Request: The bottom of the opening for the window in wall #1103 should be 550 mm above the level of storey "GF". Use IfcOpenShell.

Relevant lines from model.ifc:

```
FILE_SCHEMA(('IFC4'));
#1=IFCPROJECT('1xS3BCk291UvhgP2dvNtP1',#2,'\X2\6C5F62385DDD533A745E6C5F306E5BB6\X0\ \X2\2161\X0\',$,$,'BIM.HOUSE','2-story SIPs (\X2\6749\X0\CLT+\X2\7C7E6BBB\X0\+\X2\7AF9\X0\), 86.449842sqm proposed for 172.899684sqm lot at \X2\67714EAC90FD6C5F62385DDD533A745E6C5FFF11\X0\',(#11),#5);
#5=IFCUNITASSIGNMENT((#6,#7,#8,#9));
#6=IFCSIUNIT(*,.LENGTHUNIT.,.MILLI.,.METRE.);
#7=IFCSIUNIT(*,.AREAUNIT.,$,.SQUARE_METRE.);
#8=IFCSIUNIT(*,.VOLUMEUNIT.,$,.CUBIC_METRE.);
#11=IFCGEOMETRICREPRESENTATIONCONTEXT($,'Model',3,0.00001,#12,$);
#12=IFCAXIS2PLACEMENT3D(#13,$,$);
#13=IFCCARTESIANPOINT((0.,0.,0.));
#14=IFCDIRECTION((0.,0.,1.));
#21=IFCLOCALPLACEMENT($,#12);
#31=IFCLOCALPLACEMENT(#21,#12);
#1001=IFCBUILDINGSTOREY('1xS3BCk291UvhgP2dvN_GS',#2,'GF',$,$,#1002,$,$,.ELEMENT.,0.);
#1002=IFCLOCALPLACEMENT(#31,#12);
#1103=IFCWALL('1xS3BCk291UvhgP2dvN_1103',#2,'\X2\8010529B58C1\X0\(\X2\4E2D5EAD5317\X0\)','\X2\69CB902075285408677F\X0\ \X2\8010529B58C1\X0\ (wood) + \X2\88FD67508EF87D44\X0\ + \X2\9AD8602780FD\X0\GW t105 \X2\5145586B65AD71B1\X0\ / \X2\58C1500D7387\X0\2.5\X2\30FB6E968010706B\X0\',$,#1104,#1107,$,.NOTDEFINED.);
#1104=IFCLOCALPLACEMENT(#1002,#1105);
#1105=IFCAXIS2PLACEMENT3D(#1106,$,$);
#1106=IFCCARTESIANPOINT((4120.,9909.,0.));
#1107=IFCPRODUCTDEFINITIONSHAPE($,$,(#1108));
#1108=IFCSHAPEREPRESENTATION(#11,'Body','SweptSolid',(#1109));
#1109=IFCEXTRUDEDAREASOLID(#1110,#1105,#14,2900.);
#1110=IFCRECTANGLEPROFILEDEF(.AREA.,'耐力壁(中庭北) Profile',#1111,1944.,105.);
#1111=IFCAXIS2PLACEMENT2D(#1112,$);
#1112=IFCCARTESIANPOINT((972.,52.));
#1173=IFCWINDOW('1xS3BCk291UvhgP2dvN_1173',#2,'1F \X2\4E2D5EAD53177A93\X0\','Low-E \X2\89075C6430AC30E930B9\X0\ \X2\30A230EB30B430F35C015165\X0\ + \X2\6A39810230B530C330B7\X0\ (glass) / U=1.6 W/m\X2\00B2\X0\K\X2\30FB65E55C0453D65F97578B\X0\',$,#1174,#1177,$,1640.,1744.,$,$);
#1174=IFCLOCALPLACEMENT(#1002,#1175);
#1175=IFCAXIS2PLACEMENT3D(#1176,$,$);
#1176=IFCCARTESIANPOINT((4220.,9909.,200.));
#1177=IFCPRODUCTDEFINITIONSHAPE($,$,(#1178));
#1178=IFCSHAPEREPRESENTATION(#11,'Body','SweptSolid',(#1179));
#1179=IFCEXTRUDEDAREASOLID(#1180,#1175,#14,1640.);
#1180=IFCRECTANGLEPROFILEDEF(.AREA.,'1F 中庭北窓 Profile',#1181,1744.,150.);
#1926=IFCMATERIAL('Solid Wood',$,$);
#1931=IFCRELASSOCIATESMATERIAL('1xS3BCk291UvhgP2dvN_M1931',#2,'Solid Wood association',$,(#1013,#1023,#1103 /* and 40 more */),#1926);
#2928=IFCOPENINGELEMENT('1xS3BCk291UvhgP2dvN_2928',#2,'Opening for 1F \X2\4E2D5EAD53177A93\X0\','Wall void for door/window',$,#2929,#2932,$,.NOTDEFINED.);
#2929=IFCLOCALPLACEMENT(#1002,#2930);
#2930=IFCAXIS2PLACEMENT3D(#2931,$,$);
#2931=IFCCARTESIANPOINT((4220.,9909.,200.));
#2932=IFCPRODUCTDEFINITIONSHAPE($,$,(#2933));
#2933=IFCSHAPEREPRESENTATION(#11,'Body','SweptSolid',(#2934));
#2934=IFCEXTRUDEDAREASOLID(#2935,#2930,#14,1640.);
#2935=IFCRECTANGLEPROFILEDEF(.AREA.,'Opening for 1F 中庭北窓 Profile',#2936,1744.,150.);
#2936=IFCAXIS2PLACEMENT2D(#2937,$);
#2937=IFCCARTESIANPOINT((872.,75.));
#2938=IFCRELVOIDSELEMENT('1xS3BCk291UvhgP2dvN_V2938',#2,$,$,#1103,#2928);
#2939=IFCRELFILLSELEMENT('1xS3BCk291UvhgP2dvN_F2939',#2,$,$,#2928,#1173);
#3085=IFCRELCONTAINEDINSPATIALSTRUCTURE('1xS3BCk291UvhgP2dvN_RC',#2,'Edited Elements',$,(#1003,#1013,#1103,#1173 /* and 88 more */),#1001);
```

```python
import numpy as np
import ifcopenshell
import ifcopenshell.api.geometry
import ifcopenshell.geom
import ifcopenshell.util.element
import ifcopenshell.util.placement
import ifcopenshell.util.shape
import ifcopenshell.util.unit

model = ifcopenshell.open("model.ifc")
unit_scale = ifcopenshell.util.unit.calculate_unit_scale(model)

window = model.by_guid("1xS3BCk291UvhgP2dvN_1173")
opening = window.FillsVoids[0].RelatingOpeningElement
storey = ifcopenshell.util.element.get_container(window, ifc_class="IfcBuildingStorey")
level = ifcopenshell.util.placement.get_local_placement(storey.ObjectPlacement)[2, 3]

# The opening's origin need not be at the sill, so measure its lowest point.
shape = ifcopenshell.geom.create_shape(ifcopenshell.geom.settings(), opening)
bottom = ifcopenshell.util.shape.get_shape_bottom_elevation(shape, shape.geometry) / unit_scale
dz = level + 0.55 / unit_scale - bottom

shift = np.array([0.0, 0.0, dz])
# The window is not placed relative to its opening, so move both.
for product in (opening, window):
    matrix = ifcopenshell.util.placement.get_local_placement(product.ObjectPlacement)
    matrix[:3, 3] += shift
    ifcopenshell.api.geometry.edit_object_placement(model, product=product, matrix=matrix, is_si=False)

print(f"moved by {dz * unit_scale:+.3f} m")

model.write("model-out.ifc")
```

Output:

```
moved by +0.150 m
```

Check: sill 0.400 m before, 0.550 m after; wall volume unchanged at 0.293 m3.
